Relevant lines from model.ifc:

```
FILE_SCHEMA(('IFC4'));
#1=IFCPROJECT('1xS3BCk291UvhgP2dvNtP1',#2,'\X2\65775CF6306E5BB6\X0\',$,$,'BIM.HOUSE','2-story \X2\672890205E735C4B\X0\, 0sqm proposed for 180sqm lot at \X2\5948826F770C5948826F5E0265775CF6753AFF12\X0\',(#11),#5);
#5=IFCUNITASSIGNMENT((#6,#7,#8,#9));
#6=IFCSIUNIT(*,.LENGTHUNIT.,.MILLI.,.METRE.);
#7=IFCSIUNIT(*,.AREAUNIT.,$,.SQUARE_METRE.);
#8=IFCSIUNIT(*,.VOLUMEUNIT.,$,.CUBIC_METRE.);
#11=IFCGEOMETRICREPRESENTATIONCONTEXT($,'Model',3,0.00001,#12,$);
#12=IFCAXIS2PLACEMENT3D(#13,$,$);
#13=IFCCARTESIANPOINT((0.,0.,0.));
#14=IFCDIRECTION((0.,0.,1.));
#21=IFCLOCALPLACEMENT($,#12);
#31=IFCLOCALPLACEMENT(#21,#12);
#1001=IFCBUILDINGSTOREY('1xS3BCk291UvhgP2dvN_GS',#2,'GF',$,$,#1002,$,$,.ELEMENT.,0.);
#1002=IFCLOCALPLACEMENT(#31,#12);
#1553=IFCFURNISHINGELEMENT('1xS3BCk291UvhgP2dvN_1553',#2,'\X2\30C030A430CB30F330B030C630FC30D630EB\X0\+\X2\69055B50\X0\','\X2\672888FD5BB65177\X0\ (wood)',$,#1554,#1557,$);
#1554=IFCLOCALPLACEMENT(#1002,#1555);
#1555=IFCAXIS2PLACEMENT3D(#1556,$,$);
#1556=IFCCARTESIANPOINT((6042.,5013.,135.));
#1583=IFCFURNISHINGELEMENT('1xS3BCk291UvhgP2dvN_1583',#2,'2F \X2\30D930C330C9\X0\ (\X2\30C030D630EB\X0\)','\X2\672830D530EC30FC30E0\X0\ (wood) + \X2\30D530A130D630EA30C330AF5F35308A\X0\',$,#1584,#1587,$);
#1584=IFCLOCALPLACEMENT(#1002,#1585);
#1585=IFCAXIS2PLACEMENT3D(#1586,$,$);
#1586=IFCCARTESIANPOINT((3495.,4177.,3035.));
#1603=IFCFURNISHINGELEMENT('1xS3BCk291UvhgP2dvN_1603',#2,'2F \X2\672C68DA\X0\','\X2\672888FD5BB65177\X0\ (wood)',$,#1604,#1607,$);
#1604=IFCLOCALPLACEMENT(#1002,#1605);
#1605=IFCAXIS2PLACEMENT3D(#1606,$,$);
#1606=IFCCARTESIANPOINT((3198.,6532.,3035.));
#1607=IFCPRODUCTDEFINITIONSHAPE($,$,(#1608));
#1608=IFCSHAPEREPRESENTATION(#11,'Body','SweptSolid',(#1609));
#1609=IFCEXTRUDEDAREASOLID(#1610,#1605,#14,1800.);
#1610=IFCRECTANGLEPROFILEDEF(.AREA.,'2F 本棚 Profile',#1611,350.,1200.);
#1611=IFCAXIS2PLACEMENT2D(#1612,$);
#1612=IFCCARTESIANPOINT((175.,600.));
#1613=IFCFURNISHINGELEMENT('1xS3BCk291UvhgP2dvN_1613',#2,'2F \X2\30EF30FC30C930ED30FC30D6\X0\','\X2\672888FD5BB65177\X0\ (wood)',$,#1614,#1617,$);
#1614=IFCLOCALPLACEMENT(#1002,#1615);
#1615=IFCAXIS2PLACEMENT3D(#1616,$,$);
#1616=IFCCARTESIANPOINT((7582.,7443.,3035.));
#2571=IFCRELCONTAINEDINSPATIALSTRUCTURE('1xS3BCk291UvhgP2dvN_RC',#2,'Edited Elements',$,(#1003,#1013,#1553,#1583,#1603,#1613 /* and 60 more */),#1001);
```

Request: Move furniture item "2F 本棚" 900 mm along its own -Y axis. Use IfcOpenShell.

```python
import ifcopenshell
import ifcopenshell.api.geometry
import ifcopenshell.util.placement
import ifcopenshell.util.unit

model = ifcopenshell.open("model.ifc")
unit_scale = ifcopenshell.util.unit.calculate_unit_scale(model)

item = model.by_guid("1xS3BCk291UvhgP2dvN_1603")
matrix = ifcopenshell.util.placement.get_local_placement(item.ObjectPlacement)
matrix[:3, 3] -= matrix[:3, 1] * 0.9 / unit_scale
ifcopenshell.api.geometry.edit_object_placement(model, product=item, matrix=matrix, is_si=False)

print(ifcopenshell.util.placement.get_local_placement(item.ObjectPlacement).round(3) + 0.0)

model.write("model_v2.ifc")
```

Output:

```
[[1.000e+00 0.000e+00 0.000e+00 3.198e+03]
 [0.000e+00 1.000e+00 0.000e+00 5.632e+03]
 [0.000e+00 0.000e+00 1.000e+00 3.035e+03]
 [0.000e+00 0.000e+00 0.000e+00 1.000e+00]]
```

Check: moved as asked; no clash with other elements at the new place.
